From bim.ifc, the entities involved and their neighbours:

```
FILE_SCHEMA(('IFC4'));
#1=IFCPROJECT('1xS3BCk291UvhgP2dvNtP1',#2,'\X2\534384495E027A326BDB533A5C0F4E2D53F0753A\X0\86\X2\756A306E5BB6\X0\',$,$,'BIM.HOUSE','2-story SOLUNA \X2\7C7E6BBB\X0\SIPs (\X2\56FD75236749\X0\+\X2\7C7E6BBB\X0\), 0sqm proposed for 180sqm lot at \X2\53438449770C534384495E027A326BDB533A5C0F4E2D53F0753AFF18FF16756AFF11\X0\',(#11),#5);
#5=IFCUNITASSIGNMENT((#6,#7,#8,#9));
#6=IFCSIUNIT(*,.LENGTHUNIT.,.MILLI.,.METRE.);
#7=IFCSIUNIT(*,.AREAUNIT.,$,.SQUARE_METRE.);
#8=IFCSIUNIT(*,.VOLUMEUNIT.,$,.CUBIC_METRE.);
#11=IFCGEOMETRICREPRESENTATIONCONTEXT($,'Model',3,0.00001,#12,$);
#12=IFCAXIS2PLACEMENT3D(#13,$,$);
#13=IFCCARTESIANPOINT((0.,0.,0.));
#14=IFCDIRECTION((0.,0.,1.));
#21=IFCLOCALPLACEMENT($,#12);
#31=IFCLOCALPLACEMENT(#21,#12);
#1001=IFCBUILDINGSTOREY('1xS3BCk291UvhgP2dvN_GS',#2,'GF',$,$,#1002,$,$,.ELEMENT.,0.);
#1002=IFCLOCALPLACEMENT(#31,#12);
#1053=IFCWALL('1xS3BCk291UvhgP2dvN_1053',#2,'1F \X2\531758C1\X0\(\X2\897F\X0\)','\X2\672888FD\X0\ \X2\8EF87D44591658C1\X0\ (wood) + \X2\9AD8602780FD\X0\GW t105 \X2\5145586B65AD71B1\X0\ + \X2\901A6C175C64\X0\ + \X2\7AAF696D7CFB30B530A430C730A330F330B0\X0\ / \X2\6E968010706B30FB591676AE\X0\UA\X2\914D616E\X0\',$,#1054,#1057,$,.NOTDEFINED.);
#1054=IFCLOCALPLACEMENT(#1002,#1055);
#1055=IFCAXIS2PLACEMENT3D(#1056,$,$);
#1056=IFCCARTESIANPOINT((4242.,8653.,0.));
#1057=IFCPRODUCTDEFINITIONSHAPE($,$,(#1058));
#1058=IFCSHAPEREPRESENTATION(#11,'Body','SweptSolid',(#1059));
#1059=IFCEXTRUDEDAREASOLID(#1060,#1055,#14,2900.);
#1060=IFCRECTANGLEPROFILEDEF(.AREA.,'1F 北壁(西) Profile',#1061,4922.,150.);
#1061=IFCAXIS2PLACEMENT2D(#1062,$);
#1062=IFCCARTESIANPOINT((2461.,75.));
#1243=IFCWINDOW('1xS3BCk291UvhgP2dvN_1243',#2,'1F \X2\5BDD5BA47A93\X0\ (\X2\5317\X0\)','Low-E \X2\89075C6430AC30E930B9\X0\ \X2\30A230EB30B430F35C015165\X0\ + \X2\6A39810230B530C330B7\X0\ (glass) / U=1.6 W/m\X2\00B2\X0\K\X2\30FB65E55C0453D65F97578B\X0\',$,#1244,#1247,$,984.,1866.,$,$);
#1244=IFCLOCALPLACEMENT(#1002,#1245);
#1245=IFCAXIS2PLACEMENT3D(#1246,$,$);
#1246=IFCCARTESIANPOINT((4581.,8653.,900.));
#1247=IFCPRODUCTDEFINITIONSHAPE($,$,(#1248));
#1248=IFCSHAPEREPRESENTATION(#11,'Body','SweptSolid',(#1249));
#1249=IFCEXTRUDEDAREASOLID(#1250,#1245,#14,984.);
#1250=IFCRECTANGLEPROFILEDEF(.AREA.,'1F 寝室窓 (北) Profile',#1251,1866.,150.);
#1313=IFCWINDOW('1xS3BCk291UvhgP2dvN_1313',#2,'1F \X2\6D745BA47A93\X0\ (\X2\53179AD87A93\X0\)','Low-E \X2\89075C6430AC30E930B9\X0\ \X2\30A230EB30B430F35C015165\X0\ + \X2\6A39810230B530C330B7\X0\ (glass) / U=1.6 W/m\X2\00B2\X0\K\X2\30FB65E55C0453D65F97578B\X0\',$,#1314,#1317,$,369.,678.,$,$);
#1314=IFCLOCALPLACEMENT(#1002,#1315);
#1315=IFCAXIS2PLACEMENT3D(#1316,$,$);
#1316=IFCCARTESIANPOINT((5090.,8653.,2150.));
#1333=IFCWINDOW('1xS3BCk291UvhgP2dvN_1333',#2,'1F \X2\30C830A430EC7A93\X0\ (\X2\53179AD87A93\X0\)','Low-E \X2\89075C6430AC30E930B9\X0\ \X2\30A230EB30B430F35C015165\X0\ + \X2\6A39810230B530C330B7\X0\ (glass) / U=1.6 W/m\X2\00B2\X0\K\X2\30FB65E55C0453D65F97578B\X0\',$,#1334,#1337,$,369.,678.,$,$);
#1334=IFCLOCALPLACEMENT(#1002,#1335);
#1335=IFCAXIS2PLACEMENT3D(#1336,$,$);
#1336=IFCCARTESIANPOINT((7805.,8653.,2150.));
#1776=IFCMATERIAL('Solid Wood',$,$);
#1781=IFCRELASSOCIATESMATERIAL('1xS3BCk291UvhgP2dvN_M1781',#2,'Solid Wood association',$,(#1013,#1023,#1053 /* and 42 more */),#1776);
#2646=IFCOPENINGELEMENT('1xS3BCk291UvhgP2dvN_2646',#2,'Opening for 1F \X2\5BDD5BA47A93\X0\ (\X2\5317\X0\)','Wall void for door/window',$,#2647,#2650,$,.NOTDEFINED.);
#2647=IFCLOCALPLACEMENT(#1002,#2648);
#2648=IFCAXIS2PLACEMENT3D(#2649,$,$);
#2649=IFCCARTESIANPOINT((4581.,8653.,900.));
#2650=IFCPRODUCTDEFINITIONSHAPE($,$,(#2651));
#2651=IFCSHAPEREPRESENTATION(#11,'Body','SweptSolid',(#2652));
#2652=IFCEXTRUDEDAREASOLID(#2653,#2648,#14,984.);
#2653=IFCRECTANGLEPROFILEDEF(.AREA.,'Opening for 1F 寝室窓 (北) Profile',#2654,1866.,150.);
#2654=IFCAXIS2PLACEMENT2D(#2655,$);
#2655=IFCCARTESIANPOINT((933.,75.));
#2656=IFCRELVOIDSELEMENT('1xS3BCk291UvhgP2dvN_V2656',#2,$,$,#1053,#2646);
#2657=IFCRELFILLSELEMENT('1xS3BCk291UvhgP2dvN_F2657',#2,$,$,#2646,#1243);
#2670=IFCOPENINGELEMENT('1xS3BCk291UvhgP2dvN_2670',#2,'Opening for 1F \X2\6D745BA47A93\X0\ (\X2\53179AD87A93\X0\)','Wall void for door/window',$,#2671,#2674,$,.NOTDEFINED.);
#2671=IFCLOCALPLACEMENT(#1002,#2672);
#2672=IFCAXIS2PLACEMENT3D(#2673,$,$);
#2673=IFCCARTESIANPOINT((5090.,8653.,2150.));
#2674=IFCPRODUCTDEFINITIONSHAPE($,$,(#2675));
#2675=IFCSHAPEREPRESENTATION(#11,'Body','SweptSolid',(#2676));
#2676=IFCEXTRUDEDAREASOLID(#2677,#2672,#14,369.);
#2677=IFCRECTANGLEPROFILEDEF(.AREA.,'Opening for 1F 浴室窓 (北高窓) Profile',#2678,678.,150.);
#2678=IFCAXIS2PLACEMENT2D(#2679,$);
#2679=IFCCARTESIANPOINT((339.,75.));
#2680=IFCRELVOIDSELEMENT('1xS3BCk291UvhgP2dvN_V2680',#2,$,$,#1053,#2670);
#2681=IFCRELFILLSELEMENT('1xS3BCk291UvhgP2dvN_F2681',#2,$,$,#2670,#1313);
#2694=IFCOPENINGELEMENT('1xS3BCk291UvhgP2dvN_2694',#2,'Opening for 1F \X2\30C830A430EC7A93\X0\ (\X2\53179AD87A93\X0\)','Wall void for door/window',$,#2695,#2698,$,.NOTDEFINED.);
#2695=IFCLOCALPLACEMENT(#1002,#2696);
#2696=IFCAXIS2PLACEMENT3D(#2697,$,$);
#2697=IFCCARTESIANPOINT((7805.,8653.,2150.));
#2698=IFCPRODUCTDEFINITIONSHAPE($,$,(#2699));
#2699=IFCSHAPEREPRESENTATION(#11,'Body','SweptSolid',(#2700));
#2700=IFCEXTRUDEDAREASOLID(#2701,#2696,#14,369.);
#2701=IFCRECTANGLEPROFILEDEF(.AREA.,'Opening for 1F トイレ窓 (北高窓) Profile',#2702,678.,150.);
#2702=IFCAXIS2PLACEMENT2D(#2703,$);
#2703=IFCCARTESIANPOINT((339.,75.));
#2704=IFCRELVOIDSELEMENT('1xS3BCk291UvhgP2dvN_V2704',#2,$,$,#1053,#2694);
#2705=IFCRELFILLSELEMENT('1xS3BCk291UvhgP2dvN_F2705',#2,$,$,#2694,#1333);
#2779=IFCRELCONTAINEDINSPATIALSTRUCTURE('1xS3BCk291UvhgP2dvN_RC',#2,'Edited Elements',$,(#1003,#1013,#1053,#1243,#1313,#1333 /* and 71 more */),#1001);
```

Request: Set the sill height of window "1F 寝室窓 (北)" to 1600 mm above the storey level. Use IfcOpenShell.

```python
import numpy as np
import ifcopenshell
import ifcopenshell.api.geometry
import ifcopenshell.geom
import ifcopenshell.util.element
import ifcopenshell.util.placement
import ifcopenshell.util.shape
import ifcopenshell.util.unit

model = ifcopenshell.open("bim.ifc")
unit_scale = ifcopenshell.util.unit.calculate_unit_scale(model)

window = model.by_guid("1xS3BCk291UvhgP2dvN_1243")
opening = window.FillsVoids[0].RelatingOpeningElement
storey = ifcopenshell.util.element.get_container(window, ifc_class="IfcBuildingStorey")
level = ifcopenshell.util.placement.get_local_placement(storey.ObjectPlacement)[2, 3]

# The opening's origin need not be at the sill, so measure its lowest point.
shape = ifcopenshell.geom.create_shape(ifcopenshell.geom.settings(), opening)
bottom = ifcopenshell.util.shape.get_shape_bottom_elevation(shape, shape.geometry) / unit_scale
dz = level + 1600.0 - bottom

shift = np.array([0.0, 0.0, dz])
# The window is not placed relative to its opening, so move both.
for product in (opening, window):
    matrix = ifcopenshell.util.placement.get_local_placement(product.ObjectPlacement)
    matrix[:3, 3] += shift
    ifcopenshell.api.geometry.edit_object_placement(model, product=product, matrix=matrix, is_si=False)

print(f"moved by {dz * unit_scale:+.3f} m")

model.write("bim-out.ifc")
```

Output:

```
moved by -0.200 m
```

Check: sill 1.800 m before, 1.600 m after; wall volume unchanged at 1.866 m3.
